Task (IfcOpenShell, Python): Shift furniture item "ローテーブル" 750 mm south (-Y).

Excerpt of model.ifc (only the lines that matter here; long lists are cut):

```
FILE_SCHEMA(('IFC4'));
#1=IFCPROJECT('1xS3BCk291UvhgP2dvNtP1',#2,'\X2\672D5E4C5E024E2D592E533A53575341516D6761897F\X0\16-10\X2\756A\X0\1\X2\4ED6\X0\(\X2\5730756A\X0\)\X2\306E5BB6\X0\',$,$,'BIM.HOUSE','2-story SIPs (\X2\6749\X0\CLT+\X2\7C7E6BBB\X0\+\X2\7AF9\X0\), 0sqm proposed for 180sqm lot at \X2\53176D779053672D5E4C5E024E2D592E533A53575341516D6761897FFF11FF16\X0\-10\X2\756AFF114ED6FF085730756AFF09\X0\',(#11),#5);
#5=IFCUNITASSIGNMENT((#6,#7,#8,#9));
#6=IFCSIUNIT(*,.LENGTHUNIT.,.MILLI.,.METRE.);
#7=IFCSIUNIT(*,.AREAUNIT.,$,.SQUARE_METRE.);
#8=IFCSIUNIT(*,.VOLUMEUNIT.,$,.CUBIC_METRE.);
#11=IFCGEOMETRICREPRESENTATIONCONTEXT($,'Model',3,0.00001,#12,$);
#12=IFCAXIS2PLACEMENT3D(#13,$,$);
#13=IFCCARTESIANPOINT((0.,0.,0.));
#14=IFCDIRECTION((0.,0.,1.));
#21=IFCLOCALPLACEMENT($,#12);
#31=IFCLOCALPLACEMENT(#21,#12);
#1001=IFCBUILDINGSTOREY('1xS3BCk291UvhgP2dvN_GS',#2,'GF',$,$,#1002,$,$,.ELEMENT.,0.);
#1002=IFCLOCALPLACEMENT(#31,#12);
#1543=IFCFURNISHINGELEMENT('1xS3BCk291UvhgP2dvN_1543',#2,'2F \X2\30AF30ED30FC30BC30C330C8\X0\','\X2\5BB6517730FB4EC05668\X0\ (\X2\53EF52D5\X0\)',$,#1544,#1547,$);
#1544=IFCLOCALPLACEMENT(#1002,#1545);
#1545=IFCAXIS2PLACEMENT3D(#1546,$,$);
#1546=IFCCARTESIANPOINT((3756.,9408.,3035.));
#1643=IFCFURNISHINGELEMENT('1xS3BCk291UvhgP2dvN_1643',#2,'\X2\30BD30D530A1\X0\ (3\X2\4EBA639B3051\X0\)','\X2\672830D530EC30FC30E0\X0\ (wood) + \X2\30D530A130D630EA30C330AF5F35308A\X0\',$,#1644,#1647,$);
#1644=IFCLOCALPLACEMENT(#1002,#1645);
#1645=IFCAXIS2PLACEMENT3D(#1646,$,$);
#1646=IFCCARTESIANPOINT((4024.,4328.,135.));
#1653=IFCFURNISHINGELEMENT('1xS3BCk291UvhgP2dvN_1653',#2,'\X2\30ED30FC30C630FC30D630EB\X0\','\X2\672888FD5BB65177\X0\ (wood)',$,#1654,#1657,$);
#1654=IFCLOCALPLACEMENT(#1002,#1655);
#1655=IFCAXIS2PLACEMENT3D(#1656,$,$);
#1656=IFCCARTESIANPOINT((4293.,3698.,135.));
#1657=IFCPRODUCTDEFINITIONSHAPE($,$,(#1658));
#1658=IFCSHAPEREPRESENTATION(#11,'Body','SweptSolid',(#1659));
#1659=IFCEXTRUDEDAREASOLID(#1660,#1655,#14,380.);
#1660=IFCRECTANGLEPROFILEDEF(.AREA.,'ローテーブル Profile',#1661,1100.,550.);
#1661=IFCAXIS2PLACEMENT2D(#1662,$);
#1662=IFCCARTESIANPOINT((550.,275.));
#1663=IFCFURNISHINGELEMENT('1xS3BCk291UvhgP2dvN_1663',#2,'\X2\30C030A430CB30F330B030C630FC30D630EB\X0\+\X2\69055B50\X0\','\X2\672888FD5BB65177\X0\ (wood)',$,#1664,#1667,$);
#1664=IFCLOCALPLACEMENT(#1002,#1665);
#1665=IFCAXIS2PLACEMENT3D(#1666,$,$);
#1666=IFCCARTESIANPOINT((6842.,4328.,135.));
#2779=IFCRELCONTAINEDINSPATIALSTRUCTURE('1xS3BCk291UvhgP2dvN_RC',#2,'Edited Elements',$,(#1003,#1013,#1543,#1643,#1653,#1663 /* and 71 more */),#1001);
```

```python
import ifcopenshell
import ifcopenshell.api.geometry
import ifcopenshell.util.placement

model = ifcopenshell.open("model.ifc")

item = model.by_guid("1xS3BCk291UvhgP2dvN_1653")
matrix = ifcopenshell.util.placement.get_local_placement(item.ObjectPlacement)
matrix[1, 3] -= 750.0
ifcopenshell.api.geometry.edit_object_placement(model, product=item, matrix=matrix, is_si=False)

print(ifcopenshell.util.placement.get_local_placement(item.ObjectPlacement).round(3) + 0.0)

model.write("model_v2.ifc")
```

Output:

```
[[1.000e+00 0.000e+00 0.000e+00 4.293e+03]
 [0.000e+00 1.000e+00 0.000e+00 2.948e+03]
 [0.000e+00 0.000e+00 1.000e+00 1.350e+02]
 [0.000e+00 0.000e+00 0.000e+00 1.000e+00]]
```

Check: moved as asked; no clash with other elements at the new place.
